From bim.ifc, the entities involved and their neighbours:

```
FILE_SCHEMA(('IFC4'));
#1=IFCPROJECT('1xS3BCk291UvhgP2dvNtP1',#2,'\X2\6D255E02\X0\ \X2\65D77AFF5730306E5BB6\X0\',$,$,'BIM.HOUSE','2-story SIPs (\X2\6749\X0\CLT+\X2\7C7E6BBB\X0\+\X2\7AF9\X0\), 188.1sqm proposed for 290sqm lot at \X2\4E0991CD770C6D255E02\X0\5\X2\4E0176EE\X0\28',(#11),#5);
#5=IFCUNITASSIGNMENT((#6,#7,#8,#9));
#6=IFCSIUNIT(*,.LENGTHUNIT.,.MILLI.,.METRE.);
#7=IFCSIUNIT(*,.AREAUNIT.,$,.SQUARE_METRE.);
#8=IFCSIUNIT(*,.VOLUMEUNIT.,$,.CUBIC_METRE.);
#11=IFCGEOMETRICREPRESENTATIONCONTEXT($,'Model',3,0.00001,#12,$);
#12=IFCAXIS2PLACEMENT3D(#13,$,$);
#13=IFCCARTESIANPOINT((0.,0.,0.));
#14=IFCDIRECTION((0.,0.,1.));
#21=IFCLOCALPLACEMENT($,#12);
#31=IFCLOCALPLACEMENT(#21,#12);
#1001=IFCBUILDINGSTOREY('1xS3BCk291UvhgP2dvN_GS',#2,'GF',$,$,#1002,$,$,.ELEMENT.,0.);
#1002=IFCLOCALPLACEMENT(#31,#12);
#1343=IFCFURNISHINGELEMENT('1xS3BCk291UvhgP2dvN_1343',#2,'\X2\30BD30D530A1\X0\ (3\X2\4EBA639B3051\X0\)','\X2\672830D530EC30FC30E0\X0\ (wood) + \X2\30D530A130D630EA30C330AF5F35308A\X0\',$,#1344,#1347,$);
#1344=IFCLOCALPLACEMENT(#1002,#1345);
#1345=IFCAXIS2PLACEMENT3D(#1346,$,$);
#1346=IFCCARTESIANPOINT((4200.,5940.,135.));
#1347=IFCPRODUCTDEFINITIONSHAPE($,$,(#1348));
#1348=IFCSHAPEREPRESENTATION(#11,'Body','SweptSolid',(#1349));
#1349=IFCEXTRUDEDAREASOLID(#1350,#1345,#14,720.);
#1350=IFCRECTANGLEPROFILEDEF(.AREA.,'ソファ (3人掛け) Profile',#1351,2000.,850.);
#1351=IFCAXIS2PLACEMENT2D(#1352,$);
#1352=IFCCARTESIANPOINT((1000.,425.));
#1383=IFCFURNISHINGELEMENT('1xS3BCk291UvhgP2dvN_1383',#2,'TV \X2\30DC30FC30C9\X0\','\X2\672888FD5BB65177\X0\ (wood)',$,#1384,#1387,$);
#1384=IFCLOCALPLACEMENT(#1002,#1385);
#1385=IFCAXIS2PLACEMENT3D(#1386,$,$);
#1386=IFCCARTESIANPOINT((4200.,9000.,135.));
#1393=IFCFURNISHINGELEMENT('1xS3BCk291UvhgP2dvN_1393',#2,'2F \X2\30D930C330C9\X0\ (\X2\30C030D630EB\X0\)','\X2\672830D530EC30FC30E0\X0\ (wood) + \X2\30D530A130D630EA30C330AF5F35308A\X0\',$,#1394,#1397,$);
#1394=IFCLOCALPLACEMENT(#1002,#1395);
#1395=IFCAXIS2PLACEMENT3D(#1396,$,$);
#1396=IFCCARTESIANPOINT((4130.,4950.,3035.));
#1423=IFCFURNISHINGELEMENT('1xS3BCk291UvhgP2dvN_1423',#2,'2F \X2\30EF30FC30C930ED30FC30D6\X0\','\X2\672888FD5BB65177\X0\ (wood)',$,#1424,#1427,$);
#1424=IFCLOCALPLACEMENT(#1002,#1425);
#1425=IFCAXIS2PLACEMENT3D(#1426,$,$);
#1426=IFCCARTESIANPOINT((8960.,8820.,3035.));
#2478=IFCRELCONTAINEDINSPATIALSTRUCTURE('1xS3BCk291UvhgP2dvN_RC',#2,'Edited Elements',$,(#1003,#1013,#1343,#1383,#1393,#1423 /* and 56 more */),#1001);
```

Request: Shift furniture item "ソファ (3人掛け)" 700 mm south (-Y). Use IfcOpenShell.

```python
import ifcopenshell
import ifcopenshell.api.geometry
import ifcopenshell.util.placement
import ifcopenshell.util.unit

model = ifcopenshell.open("bim.ifc")
unit_scale = ifcopenshell.util.unit.calculate_unit_scale(model)

item = model.by_id(1343)
matrix = ifcopenshell.util.placement.get_local_placement(item.ObjectPlacement)
matrix[1, 3] -= 0.7 / unit_scale
ifcopenshell.api.geometry.edit_object_placement(model, product=item, matrix=matrix, is_si=False)

print(ifcopenshell.util.placement.get_local_placement(item.ObjectPlacement).round(3) + 0.0)

model.write("bim_rev.ifc")
```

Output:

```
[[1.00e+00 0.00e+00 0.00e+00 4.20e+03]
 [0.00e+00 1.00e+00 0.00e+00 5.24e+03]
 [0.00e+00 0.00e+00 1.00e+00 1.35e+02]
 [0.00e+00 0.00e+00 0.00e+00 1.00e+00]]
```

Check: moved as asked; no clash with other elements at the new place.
